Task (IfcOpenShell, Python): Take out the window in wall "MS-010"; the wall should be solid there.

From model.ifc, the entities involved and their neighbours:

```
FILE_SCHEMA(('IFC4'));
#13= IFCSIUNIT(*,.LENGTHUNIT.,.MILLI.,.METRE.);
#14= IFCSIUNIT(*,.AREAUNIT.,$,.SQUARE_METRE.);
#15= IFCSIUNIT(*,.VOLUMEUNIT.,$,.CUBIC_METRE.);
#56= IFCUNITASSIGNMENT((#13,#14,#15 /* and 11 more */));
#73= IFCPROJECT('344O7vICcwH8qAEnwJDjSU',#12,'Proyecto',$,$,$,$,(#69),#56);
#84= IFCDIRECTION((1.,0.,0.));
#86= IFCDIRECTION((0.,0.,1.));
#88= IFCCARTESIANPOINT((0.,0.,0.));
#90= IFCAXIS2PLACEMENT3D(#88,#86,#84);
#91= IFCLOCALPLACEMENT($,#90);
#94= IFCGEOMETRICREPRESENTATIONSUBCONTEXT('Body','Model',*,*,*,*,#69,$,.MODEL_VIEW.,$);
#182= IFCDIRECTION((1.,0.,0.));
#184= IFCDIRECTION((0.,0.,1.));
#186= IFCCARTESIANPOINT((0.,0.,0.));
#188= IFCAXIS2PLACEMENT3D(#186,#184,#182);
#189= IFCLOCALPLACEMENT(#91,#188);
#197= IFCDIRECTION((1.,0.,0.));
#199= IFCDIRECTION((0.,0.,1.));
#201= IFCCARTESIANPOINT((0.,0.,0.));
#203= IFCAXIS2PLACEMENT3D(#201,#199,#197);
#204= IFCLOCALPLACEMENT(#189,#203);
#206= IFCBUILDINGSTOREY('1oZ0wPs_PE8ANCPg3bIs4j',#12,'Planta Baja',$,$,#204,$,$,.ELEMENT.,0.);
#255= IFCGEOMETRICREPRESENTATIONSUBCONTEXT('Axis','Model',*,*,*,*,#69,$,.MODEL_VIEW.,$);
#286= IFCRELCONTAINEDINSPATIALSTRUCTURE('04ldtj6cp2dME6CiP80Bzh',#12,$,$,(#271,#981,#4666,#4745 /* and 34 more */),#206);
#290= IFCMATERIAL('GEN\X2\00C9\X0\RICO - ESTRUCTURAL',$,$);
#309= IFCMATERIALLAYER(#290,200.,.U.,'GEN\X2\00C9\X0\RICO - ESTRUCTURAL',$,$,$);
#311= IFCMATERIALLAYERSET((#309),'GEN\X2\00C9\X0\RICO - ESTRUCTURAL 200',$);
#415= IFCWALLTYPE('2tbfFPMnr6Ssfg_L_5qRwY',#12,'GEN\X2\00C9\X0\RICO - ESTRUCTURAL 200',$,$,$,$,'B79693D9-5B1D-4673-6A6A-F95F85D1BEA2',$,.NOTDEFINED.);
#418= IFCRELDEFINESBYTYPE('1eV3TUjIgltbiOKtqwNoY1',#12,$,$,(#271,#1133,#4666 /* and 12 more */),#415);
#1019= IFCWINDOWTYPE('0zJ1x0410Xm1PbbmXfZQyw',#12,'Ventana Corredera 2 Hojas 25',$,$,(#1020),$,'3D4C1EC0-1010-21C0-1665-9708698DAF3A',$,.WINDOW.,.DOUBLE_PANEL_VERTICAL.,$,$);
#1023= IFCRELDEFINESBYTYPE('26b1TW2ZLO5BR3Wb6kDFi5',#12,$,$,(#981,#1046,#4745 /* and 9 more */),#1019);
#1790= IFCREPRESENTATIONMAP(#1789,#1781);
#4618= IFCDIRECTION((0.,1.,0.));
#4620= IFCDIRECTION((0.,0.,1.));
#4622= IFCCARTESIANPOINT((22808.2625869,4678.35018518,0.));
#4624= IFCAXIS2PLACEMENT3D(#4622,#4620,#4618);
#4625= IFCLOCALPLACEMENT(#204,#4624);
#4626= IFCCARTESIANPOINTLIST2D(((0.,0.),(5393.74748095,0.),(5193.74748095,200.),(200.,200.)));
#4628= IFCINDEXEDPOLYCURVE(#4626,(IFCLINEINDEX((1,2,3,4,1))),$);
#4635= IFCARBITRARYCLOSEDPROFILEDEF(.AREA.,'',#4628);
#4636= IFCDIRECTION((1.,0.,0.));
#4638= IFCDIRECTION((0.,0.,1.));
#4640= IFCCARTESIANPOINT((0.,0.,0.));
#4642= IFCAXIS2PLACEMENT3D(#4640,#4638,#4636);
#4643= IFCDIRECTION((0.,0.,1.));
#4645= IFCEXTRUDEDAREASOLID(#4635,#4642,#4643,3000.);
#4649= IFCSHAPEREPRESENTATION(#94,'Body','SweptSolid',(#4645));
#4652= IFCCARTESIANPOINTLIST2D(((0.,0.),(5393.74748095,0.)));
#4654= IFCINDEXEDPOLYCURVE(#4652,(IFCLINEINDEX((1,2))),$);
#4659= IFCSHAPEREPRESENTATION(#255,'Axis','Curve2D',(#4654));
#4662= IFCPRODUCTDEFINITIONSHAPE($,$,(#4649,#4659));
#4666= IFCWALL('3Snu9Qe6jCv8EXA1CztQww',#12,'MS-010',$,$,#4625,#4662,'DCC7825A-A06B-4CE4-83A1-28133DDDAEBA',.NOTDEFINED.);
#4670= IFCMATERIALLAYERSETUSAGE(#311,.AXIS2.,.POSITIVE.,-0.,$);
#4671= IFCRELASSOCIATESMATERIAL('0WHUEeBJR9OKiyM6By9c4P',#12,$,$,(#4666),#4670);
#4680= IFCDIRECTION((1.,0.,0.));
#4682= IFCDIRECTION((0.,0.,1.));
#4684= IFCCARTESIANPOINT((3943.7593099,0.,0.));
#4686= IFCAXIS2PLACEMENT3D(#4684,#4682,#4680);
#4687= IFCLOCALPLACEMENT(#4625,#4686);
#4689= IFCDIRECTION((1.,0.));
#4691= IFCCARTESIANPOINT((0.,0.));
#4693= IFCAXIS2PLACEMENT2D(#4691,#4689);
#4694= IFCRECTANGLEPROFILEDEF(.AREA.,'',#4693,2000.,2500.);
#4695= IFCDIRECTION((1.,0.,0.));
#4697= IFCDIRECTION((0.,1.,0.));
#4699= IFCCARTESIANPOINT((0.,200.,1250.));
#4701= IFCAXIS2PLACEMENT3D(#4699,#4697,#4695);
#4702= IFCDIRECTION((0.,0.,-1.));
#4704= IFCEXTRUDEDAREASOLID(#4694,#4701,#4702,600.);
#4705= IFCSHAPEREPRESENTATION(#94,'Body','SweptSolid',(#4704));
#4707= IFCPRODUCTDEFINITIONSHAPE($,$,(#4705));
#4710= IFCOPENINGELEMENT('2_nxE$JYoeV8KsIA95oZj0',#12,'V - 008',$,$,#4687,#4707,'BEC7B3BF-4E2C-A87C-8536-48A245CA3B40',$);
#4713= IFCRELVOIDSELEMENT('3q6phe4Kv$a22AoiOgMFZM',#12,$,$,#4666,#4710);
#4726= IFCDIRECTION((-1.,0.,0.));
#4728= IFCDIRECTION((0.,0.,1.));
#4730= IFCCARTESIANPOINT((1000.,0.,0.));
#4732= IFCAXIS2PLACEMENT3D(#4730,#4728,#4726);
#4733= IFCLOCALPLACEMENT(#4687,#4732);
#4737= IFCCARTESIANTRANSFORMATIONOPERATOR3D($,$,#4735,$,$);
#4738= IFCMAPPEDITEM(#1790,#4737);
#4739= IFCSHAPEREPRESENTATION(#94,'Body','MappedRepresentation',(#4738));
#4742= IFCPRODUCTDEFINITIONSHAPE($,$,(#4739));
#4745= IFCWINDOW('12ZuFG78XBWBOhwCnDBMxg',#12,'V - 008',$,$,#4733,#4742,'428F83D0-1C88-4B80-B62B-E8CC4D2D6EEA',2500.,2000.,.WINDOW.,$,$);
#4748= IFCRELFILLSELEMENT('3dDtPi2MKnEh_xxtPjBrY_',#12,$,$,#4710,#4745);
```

```python
import ifcopenshell
import ifcopenshell.api.feature
import ifcopenshell.api.root
import ifcopenshell.geom
import ifcopenshell.util.shape

model = ifcopenshell.open("model.ifc")
settings = ifcopenshell.geom.settings()


def volume(element):
    """Net volume in cubic metres, openings subtracted."""
    shape = ifcopenshell.geom.create_shape(settings, element)
    return ifcopenshell.util.shape.get_volume(shape.geometry)


window = model.by_guid("12ZuFG78XBWBOhwCnDBMxg")
opening = window.FillsVoids[0].RelatingOpeningElement
wall = opening.VoidsElements[0].RelatingBuildingElement
before = volume(wall)

ifcopenshell.api.root.remove_product(model, product=window)
ifcopenshell.api.feature.remove_feature(model, feature=opening)

after = volume(wall)

print(f"wall volume {before:.3f} -> {after:.3f} m3")

model.write("model_edited.ifc")
```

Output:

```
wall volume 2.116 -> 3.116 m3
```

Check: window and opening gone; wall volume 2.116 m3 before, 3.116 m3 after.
